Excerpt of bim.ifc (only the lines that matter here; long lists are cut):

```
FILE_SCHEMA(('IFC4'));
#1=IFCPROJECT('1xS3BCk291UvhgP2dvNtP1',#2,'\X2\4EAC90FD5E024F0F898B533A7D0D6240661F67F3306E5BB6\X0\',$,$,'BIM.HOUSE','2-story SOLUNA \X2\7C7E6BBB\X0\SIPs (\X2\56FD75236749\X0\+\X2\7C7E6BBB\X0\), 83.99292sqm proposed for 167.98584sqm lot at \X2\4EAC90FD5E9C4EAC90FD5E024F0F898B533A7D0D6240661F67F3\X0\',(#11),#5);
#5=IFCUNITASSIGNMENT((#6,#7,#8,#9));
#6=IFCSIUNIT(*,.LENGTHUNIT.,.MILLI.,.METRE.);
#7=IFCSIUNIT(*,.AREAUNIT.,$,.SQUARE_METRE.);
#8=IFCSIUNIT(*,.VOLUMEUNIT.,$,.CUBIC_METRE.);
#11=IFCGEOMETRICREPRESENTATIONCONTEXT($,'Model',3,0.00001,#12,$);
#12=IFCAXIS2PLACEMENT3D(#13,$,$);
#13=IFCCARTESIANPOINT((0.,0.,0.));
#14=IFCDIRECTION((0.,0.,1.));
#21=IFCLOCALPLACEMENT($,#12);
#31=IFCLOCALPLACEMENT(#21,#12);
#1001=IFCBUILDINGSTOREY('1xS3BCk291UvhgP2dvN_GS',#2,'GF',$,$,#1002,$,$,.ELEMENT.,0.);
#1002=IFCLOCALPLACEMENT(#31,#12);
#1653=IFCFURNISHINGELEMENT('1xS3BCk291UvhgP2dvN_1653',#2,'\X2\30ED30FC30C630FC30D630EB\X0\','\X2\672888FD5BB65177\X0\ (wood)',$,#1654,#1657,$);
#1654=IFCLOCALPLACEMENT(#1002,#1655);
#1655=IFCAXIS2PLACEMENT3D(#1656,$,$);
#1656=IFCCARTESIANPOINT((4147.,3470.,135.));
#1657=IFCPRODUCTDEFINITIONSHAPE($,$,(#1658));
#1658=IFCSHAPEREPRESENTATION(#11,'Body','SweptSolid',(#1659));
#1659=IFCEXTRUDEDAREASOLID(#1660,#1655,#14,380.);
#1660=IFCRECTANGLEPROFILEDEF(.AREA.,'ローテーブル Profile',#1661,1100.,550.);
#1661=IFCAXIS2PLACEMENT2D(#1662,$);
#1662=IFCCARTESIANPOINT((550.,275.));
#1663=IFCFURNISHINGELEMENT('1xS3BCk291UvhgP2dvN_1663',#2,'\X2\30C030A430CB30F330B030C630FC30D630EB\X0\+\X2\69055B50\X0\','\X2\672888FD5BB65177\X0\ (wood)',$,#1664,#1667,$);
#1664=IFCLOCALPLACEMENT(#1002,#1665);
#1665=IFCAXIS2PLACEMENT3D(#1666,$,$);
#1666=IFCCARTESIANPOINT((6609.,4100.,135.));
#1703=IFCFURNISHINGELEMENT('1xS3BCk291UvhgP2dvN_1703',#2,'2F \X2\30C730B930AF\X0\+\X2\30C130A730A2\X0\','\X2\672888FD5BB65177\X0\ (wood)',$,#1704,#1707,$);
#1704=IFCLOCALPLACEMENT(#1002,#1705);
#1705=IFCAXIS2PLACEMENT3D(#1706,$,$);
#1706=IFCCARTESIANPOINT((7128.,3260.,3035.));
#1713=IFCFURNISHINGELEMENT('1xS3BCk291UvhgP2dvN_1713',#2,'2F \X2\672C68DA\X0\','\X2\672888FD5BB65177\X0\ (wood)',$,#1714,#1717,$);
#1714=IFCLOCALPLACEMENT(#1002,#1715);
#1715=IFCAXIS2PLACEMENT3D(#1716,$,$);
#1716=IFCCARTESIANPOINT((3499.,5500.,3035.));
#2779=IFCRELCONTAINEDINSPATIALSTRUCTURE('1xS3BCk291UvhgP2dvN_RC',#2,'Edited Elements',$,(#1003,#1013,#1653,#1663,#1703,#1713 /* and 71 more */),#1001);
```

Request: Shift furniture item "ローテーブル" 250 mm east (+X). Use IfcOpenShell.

```python
import ifcopenshell
import ifcopenshell.api.geometry
import ifcopenshell.util.placement
import ifcopenshell.util.unit

model = ifcopenshell.open("bim.ifc")
unit_scale = ifcopenshell.util.unit.calculate_unit_scale(model)

item = model.by_guid("1xS3BCk291UvhgP2dvN_1653")
matrix = ifcopenshell.util.placement.get_local_placement(item.ObjectPlacement)
matrix[0, 3] += 0.25 / unit_scale
ifcopenshell.api.geometry.edit_object_placement(model, product=item, matrix=matrix, is_si=False)

print(ifcopenshell.util.placement.get_local_placement(item.ObjectPlacement).round(3) + 0.0)

model.write("bim_edited.ifc")
```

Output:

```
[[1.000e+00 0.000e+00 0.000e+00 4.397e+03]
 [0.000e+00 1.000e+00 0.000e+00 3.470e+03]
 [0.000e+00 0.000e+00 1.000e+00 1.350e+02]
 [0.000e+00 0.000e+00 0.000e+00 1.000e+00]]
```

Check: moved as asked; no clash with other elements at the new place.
